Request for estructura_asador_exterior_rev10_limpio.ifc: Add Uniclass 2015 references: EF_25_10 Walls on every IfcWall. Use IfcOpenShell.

First a look at what the model holds.

```python
import ifcopenshell

model = ifcopenshell.open("estructura_asador_exterior_rev10_limpio.ifc")
print(model.schema)
print("classifications:", [c.Name for c in model.by_type("IfcClassification")])
for ifc_class in ("IfcDoor", "IfcRoof", "IfcStair", "IfcWall", "IfcWindow"):
    print(ifc_class, len(model.by_type(ifc_class)))
```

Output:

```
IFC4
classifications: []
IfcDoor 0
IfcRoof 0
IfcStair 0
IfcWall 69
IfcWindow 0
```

```python
import ifcopenshell
import ifcopenshell.api.classification

model = ifcopenshell.open("estructura_asador_exterior_rev10_limpio.ifc")

system = ifcopenshell.api.classification.add_classification(model, classification="Uniclass 2015")

codes = {
    "IfcWall": ("EF_25_10", "Walls"),
}
for ifc_class, (code, name) in codes.items():
    products = model.by_type(ifc_class)
    ifcopenshell.api.classification.add_reference(
        model, products=products, classification=system, identification=code, name=name
    )
    print(code, len(products))

model.write("estructura_asador_exterior_rev10_limpio_updated.ifc")
```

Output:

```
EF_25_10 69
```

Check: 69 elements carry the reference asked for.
